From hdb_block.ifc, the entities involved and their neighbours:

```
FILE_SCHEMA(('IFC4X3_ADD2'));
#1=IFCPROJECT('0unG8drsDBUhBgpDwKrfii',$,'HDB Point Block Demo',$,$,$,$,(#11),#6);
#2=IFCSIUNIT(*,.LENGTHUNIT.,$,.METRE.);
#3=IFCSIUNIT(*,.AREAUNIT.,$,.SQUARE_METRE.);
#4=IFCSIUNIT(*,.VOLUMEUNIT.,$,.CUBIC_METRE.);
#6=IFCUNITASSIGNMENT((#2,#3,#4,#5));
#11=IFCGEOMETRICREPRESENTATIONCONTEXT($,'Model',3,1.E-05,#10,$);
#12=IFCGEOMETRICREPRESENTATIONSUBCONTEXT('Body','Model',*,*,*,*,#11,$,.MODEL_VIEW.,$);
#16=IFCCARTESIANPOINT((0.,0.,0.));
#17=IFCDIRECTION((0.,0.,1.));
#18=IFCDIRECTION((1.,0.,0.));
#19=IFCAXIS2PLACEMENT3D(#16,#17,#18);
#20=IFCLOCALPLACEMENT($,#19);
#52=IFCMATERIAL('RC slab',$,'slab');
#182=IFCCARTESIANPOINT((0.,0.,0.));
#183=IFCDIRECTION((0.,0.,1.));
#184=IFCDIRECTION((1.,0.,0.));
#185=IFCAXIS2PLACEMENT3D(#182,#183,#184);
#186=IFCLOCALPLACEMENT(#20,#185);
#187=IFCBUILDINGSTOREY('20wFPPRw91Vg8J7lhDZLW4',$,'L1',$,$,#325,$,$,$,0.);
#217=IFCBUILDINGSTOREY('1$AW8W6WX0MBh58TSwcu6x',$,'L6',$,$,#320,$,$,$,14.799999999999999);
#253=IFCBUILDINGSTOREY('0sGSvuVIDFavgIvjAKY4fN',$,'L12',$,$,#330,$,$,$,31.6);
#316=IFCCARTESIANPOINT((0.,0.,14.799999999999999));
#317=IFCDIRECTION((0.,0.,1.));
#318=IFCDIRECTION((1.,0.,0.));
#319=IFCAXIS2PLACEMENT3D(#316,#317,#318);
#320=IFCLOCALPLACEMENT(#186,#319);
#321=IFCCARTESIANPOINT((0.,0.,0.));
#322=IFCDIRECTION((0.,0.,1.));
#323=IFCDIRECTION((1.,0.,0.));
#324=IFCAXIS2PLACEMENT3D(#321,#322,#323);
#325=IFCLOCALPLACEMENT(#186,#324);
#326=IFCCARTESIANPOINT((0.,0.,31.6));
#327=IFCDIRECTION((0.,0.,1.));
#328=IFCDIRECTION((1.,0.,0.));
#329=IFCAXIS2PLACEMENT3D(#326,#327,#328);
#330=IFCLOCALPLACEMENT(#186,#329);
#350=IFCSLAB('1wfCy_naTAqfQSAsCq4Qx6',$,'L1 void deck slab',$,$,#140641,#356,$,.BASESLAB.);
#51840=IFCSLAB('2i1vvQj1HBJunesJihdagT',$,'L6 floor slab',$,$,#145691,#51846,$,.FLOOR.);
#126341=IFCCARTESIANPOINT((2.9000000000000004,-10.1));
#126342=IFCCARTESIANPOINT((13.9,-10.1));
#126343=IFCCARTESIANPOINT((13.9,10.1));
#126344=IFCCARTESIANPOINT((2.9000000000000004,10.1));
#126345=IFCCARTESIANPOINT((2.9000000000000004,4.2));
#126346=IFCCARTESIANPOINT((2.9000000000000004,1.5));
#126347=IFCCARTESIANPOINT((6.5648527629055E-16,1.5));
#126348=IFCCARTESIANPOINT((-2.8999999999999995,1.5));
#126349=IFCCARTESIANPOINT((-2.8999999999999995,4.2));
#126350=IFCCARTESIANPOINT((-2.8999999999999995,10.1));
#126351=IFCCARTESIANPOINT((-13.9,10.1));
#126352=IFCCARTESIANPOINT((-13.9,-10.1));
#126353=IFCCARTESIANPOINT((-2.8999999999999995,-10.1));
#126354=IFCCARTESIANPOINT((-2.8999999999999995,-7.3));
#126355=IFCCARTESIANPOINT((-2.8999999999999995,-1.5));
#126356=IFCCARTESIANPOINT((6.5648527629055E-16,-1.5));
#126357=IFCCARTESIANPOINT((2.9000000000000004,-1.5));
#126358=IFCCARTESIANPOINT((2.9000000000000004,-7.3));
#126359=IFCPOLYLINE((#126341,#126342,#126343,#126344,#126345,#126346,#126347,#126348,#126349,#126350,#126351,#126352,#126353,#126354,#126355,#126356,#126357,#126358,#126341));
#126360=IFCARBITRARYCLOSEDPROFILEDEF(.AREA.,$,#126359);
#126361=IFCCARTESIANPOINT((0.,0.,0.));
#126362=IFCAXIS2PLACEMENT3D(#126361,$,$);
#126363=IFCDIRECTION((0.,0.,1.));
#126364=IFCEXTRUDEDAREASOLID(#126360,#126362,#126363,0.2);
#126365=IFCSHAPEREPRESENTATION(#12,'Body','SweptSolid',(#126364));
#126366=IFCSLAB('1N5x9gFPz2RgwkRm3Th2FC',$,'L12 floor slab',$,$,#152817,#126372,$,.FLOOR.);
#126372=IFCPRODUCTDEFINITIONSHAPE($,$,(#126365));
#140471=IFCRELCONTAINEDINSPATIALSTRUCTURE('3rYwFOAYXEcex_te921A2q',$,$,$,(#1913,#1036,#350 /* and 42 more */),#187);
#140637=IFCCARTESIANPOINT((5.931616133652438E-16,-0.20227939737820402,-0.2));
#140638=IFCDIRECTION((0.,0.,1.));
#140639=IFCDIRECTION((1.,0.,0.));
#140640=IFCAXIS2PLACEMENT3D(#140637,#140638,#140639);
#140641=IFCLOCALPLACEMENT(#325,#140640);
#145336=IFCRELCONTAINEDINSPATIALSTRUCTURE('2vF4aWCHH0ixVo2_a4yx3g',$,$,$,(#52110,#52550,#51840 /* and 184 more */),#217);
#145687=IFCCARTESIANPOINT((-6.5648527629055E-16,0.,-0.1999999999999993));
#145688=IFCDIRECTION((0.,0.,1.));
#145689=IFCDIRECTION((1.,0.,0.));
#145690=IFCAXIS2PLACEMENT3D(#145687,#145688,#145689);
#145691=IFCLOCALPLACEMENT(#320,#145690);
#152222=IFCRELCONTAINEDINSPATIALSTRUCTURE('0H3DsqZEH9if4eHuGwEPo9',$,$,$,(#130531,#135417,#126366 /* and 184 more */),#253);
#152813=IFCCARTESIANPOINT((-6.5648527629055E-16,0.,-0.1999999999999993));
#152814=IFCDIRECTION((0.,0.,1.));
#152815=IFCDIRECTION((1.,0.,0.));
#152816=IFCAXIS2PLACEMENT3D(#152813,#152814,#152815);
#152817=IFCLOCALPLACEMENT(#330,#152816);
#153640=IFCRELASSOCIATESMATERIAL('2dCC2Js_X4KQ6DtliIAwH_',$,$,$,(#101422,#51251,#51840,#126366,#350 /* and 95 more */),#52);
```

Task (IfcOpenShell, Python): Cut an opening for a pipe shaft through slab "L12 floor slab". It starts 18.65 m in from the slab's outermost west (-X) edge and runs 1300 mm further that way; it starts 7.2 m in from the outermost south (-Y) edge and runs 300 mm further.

```python
import numpy as np
import ifcopenshell
import ifcopenshell.api.feature
import ifcopenshell.api.geometry
import ifcopenshell.api.root
import ifcopenshell.geom
import ifcopenshell.util.placement
import ifcopenshell.util.representation
import ifcopenshell.util.shape
import ifcopenshell.util.unit

model = ifcopenshell.open("hdb_block.ifc")
unit_scale = ifcopenshell.util.unit.calculate_unit_scale(model)
settings = ifcopenshell.geom.settings()


def volume(element):
    """Net volume in cubic metres, openings subtracted."""
    shape = ifcopenshell.geom.create_shape(settings, element)
    return ifcopenshell.util.shape.get_volume(shape.geometry)


slab = model.by_guid("1N5x9gFPz2RgwkRm3Th2FC")
before = volume(slab)

# Extent in the slab's own axes, in metres. The edges named are its -X and -Y sides.
slab_shape = ifcopenshell.geom.create_shape(settings, slab)
vertices = ifcopenshell.util.shape.get_vertices(slab_shape.geometry)
x_min, y_min, bottom = vertices.min(axis=0)
top = vertices[:, 2].max()

opening = ifcopenshell.api.root.create_entity(model, ifc_class="IfcOpeningElement", name="Pipe shaft opening", predefined_type="OPENING")
context = ifcopenshell.util.representation.get_context(model, "Model", "Body", "MODEL_VIEW")
width, depth = 1.3, 0.3
outline = [(0.0, 0.0), (width, 0.0), (width, depth), (0.0, depth), (0.0, 0.0)]
# Overshoot both faces by 50 mm so the cut is clean.
shape = ifcopenshell.api.geometry.add_slab_representation(
    model, context=context, depth=top - bottom + 0.1, polyline=outline
)
ifcopenshell.api.geometry.assign_representation(model, product=opening, representation=shape)

matrix = ifcopenshell.util.placement.get_local_placement(slab.ObjectPlacement)
matrix[:, 3] = matrix @ np.append(np.array([x_min + 18.65, y_min + 7.2, bottom - 0.05]) / unit_scale, 1.0)
ifcopenshell.api.geometry.edit_object_placement(model, product=opening, matrix=matrix, is_si=False)
ifcopenshell.api.feature.add_feature(model, feature=opening, element=slab)

after = volume(slab)

print(f"slab volume {before:.3f} -> {after:.3f} m3")

model.write("hdb_block_v2.ifc")
```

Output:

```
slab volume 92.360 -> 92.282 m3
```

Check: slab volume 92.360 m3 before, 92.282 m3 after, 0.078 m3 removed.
